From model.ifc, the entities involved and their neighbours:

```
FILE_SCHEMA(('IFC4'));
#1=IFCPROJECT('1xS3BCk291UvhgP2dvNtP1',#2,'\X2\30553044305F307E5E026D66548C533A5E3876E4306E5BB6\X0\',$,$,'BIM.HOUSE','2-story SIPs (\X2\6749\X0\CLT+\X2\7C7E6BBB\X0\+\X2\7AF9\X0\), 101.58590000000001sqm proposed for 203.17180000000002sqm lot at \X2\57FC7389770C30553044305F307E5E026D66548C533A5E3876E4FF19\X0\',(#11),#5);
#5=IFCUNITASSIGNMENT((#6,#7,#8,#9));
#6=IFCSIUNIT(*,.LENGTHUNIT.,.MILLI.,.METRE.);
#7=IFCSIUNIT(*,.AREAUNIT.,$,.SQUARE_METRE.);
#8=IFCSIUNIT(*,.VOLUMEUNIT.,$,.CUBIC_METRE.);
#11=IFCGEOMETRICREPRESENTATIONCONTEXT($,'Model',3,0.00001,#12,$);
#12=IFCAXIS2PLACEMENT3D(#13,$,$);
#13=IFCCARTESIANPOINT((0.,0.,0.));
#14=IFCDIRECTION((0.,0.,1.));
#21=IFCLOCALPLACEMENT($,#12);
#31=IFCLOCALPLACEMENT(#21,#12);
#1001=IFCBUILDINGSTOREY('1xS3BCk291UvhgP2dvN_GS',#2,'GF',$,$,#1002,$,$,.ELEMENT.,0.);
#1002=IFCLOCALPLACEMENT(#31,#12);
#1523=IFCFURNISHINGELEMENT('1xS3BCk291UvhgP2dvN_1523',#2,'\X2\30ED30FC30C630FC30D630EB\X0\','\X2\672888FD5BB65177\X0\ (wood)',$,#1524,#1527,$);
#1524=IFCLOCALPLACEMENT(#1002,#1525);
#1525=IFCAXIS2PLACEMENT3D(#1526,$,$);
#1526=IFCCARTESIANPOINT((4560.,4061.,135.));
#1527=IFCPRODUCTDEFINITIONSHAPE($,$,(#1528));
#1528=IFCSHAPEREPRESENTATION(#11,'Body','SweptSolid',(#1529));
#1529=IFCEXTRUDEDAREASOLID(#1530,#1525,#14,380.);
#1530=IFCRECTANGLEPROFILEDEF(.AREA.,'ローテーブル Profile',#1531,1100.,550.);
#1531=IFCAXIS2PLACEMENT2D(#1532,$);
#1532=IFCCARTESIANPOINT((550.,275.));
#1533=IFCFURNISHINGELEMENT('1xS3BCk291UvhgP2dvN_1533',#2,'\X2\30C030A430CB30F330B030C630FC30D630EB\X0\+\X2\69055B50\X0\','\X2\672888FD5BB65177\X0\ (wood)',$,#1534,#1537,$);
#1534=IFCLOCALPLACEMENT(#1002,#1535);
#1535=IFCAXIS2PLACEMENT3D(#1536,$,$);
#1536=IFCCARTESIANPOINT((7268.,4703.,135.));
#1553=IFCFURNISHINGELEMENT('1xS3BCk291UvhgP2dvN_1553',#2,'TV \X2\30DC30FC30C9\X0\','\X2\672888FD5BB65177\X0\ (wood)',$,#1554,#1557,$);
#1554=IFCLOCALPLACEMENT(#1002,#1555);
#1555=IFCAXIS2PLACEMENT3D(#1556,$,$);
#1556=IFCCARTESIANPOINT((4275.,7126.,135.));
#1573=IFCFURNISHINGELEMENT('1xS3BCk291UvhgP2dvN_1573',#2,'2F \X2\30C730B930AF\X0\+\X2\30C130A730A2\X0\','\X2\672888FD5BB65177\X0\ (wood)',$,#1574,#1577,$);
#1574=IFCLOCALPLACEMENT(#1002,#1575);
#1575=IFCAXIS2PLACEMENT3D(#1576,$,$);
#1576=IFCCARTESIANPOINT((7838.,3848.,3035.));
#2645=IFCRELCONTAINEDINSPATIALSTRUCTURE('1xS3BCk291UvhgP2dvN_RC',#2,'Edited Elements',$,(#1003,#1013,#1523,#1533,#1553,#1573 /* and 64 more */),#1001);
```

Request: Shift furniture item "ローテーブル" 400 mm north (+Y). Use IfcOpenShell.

```python
import ifcopenshell
import ifcopenshell.api.geometry
import ifcopenshell.util.placement
import ifcopenshell.util.unit

model = ifcopenshell.open("model.ifc")
unit_scale = ifcopenshell.util.unit.calculate_unit_scale(model)

item = model.by_guid("1xS3BCk291UvhgP2dvN_1523")
matrix = ifcopenshell.util.placement.get_local_placement(item.ObjectPlacement)
matrix[1, 3] += 0.4 / unit_scale
ifcopenshell.api.geometry.edit_object_placement(model, product=item, matrix=matrix, is_si=False)

print(ifcopenshell.util.placement.get_local_placement(item.ObjectPlacement).round(3) + 0.0)

model.write("model_rev.ifc")
```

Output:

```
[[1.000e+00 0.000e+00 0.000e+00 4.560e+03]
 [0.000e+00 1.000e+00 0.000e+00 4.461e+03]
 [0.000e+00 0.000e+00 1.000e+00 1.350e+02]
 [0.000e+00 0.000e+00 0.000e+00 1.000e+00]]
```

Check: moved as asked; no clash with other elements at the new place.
